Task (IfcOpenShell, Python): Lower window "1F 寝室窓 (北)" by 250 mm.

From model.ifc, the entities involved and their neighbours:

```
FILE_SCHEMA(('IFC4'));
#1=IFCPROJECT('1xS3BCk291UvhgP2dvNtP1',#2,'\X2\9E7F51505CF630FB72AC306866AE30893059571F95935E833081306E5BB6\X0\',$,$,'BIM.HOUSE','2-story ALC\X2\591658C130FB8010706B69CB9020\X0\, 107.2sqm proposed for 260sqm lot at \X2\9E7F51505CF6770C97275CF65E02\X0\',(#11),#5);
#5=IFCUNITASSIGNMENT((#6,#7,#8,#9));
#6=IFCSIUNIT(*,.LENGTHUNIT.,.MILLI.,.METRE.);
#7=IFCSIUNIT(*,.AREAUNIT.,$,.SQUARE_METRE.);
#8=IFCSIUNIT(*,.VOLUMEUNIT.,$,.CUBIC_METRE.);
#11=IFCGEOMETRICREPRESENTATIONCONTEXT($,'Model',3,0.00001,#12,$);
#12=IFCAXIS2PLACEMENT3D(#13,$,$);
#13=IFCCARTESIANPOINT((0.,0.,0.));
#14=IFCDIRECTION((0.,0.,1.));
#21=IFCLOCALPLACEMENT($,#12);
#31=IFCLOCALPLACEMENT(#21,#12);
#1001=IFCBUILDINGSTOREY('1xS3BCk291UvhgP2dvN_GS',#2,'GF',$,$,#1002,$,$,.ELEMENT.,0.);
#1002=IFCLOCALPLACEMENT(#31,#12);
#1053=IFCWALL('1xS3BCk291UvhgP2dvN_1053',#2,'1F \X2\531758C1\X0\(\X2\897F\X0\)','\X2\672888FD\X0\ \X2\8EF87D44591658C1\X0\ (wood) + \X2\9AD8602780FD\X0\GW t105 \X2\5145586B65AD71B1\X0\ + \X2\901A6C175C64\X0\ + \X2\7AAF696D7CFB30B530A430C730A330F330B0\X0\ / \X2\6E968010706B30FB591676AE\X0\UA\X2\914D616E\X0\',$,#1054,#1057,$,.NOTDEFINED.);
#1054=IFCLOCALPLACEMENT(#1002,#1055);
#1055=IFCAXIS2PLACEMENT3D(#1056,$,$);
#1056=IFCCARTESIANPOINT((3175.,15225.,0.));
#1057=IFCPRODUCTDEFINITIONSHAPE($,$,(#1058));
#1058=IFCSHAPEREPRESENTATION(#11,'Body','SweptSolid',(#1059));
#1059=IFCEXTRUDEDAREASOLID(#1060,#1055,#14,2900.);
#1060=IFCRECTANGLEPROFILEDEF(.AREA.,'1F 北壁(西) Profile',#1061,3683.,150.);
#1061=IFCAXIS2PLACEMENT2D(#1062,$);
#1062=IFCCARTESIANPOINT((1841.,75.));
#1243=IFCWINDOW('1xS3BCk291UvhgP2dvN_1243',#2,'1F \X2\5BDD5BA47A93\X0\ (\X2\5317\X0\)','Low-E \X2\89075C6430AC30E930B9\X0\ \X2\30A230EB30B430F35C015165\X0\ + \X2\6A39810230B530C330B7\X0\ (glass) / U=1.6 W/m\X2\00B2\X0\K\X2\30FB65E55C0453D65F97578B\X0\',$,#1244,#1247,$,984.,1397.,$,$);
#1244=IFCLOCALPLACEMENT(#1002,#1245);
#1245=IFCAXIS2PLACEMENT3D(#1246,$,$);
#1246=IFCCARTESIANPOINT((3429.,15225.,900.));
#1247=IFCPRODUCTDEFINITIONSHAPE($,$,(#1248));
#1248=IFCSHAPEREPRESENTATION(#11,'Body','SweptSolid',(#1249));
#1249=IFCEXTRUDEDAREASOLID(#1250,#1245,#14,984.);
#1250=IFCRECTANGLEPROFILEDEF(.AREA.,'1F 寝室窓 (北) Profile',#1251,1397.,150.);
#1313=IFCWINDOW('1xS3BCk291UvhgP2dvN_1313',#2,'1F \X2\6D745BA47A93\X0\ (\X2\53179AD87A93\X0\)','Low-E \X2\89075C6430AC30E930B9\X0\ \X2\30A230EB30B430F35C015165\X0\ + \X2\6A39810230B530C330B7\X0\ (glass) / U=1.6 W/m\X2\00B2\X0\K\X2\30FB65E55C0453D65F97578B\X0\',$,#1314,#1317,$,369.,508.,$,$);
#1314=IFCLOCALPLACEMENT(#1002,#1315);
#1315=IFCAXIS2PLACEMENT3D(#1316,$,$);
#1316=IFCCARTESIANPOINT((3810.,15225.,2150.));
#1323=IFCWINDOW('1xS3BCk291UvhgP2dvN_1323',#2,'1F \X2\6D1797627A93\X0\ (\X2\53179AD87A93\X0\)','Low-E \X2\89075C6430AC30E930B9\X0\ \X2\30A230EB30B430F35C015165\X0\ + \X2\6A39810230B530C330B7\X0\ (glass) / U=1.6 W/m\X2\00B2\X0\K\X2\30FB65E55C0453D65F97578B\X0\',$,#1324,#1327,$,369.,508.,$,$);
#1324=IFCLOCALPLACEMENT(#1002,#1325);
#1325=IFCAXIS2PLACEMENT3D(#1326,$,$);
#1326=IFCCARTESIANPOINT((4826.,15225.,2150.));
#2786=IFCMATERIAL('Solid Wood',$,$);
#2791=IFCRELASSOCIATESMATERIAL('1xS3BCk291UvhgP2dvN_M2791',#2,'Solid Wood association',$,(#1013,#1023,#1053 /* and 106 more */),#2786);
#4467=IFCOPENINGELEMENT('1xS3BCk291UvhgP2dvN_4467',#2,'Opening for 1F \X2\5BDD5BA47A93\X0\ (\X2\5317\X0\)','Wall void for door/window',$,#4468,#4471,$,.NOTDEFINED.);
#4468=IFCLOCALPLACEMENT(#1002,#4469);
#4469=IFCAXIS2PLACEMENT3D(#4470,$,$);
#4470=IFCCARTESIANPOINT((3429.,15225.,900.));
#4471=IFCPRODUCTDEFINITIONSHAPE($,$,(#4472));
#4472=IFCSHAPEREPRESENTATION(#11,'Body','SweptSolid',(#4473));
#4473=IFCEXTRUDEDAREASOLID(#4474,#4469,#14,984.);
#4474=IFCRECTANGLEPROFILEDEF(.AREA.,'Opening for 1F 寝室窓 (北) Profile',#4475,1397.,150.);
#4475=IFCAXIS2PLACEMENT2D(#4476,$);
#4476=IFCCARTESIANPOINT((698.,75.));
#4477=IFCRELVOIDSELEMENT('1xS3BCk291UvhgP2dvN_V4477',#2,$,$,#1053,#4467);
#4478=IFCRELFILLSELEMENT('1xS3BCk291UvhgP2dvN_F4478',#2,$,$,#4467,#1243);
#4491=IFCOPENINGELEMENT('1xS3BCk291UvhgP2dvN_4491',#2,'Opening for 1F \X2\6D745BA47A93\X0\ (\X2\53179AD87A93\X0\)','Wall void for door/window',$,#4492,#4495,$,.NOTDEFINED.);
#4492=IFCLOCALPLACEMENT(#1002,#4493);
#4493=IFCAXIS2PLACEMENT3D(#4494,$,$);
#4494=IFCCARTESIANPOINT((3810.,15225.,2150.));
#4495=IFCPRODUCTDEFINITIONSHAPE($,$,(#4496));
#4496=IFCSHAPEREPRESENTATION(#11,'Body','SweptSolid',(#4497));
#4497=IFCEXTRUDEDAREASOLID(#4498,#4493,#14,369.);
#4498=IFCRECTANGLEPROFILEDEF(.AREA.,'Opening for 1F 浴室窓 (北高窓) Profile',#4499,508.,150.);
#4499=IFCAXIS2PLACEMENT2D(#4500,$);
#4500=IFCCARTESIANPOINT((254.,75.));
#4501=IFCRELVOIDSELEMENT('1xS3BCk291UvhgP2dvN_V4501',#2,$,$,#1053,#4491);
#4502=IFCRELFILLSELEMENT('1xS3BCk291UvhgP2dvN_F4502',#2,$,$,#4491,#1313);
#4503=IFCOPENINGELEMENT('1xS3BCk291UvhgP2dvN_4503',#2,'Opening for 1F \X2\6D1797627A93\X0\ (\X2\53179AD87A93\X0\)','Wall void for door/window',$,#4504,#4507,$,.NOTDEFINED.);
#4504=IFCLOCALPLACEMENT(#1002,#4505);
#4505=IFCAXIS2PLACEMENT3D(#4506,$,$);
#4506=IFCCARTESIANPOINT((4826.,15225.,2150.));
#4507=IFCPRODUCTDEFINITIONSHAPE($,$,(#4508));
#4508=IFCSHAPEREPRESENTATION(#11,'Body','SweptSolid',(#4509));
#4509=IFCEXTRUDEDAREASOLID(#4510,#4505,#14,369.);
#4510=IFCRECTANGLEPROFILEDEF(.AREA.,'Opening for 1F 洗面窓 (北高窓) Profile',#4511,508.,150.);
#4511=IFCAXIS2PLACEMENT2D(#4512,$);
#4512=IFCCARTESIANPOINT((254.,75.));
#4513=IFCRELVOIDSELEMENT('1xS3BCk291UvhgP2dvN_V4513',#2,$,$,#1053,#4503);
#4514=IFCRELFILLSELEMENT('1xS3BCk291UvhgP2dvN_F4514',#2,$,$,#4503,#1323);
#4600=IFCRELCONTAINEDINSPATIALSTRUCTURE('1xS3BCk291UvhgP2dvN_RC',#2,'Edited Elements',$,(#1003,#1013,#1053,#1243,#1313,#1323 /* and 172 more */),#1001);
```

```python
import numpy as np
import ifcopenshell
import ifcopenshell.api.geometry
import ifcopenshell.util.placement
import ifcopenshell.util.unit

model = ifcopenshell.open("model.ifc")
unit_scale = ifcopenshell.util.unit.calculate_unit_scale(model)

window = model.by_guid("1xS3BCk291UvhgP2dvN_1243")
opening = window.FillsVoids[0].RelatingOpeningElement
dz = -0.25 / unit_scale

shift = np.array([0.0, 0.0, dz])
# The window is not placed relative to its opening, so move both.
for product in (opening, window):
    matrix = ifcopenshell.util.placement.get_local_placement(product.ObjectPlacement)
    matrix[:3, 3] += shift
    ifcopenshell.api.geometry.edit_object_placement(model, product=product, matrix=matrix, is_si=False)

print(f"moved by {dz * unit_scale:+.3f} m")

model.write("model_updated.ifc")
```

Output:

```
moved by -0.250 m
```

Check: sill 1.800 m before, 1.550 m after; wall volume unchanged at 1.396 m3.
